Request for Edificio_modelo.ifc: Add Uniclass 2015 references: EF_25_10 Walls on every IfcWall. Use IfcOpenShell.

First a look at what the model holds.

```python
import ifcopenshell

model = ifcopenshell.open("Edificio_modelo.ifc")
print(model.schema)
print("classifications:", [c.Name for c in model.by_type("IfcClassification")])
for ifc_class in ("IfcDoor", "IfcRoof", "IfcStair", "IfcWall", "IfcWindow"):
    print(ifc_class, len(model.by_type(ifc_class)))
```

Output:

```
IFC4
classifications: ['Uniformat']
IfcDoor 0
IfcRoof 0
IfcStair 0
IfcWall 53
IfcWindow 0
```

```python
import ifcopenshell
import ifcopenshell.api.classification

model = ifcopenshell.open("Edificio_modelo.ifc")

system = ifcopenshell.api.classification.add_classification(model, classification="Uniclass 2015")

codes = {
    "IfcWall": ("EF_25_10", "Walls"),
}
for ifc_class, (code, name) in codes.items():
    products = model.by_type(ifc_class)
    ifcopenshell.api.classification.add_reference(
        model, products=products, classification=system, identification=code, name=name
    )
    print(code, len(products))

model.write("Edificio_modelo_edited.ifc")
```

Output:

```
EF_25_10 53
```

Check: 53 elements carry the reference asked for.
